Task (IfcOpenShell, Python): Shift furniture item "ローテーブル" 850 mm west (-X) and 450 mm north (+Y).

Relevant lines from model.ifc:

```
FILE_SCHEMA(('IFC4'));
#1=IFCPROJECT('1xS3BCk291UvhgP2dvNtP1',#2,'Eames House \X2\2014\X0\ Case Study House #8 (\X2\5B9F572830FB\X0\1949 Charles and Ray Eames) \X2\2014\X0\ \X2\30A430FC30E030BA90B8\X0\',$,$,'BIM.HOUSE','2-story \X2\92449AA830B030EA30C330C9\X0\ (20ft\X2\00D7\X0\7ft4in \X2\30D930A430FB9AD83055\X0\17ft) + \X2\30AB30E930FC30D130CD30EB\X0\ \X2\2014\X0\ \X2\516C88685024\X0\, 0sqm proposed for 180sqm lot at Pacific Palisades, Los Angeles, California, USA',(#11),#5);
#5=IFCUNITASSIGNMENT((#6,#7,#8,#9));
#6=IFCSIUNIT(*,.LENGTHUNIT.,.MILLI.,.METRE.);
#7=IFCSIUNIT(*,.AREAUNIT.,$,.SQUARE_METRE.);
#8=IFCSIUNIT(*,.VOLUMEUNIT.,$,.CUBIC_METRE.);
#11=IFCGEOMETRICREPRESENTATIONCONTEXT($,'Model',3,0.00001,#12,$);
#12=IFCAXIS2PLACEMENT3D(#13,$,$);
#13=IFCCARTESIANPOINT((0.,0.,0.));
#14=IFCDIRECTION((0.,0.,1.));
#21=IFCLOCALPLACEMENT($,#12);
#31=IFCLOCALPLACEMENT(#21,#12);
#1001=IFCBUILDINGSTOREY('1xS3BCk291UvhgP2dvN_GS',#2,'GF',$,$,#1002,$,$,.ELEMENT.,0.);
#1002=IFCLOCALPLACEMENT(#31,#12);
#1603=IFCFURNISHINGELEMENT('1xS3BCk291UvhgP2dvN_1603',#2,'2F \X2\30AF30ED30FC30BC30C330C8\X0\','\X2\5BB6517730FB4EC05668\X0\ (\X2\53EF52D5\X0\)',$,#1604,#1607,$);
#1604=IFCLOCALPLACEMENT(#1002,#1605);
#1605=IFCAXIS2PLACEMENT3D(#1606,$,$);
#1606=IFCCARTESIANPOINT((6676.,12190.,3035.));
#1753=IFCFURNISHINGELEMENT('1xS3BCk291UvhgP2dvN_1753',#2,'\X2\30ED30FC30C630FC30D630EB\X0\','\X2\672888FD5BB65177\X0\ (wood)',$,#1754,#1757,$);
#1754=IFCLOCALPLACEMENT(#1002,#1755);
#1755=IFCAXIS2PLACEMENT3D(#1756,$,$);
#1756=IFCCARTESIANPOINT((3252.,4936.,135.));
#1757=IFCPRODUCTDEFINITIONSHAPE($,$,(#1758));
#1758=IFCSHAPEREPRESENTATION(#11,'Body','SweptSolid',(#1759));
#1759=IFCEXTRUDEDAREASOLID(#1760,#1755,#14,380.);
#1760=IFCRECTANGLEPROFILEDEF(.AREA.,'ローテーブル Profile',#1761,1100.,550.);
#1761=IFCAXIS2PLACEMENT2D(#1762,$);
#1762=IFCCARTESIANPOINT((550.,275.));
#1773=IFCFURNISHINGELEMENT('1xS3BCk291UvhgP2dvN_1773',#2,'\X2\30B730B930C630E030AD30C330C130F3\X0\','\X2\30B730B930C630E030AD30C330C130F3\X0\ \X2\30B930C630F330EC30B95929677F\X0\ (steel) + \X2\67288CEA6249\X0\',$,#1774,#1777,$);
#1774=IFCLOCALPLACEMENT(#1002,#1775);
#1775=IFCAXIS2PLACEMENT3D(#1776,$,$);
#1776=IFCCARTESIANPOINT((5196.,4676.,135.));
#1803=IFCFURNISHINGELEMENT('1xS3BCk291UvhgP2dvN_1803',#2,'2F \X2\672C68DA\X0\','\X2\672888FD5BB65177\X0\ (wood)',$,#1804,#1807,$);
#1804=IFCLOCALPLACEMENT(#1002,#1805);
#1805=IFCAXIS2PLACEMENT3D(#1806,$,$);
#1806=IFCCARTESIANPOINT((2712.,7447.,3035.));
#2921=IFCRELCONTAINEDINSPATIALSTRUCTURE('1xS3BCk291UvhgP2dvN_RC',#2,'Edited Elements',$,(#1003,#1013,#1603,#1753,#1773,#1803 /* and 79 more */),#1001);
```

```python
import ifcopenshell
import ifcopenshell.api.geometry
import ifcopenshell.util.placement

model = ifcopenshell.open("model.ifc")

item = model.by_guid("1xS3BCk291UvhgP2dvN_1753")
matrix = ifcopenshell.util.placement.get_local_placement(item.ObjectPlacement)
matrix[0, 3] -= 850.0
matrix[1, 3] += 450.0
ifcopenshell.api.geometry.edit_object_placement(model, product=item, matrix=matrix, is_si=False)

print(ifcopenshell.util.placement.get_local_placement(item.ObjectPlacement).round(3) + 0.0)

model.write("model-out.ifc")
```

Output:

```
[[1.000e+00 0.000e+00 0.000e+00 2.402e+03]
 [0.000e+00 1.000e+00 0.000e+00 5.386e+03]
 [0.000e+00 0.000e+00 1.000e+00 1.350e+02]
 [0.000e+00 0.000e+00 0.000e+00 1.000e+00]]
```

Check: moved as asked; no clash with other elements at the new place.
